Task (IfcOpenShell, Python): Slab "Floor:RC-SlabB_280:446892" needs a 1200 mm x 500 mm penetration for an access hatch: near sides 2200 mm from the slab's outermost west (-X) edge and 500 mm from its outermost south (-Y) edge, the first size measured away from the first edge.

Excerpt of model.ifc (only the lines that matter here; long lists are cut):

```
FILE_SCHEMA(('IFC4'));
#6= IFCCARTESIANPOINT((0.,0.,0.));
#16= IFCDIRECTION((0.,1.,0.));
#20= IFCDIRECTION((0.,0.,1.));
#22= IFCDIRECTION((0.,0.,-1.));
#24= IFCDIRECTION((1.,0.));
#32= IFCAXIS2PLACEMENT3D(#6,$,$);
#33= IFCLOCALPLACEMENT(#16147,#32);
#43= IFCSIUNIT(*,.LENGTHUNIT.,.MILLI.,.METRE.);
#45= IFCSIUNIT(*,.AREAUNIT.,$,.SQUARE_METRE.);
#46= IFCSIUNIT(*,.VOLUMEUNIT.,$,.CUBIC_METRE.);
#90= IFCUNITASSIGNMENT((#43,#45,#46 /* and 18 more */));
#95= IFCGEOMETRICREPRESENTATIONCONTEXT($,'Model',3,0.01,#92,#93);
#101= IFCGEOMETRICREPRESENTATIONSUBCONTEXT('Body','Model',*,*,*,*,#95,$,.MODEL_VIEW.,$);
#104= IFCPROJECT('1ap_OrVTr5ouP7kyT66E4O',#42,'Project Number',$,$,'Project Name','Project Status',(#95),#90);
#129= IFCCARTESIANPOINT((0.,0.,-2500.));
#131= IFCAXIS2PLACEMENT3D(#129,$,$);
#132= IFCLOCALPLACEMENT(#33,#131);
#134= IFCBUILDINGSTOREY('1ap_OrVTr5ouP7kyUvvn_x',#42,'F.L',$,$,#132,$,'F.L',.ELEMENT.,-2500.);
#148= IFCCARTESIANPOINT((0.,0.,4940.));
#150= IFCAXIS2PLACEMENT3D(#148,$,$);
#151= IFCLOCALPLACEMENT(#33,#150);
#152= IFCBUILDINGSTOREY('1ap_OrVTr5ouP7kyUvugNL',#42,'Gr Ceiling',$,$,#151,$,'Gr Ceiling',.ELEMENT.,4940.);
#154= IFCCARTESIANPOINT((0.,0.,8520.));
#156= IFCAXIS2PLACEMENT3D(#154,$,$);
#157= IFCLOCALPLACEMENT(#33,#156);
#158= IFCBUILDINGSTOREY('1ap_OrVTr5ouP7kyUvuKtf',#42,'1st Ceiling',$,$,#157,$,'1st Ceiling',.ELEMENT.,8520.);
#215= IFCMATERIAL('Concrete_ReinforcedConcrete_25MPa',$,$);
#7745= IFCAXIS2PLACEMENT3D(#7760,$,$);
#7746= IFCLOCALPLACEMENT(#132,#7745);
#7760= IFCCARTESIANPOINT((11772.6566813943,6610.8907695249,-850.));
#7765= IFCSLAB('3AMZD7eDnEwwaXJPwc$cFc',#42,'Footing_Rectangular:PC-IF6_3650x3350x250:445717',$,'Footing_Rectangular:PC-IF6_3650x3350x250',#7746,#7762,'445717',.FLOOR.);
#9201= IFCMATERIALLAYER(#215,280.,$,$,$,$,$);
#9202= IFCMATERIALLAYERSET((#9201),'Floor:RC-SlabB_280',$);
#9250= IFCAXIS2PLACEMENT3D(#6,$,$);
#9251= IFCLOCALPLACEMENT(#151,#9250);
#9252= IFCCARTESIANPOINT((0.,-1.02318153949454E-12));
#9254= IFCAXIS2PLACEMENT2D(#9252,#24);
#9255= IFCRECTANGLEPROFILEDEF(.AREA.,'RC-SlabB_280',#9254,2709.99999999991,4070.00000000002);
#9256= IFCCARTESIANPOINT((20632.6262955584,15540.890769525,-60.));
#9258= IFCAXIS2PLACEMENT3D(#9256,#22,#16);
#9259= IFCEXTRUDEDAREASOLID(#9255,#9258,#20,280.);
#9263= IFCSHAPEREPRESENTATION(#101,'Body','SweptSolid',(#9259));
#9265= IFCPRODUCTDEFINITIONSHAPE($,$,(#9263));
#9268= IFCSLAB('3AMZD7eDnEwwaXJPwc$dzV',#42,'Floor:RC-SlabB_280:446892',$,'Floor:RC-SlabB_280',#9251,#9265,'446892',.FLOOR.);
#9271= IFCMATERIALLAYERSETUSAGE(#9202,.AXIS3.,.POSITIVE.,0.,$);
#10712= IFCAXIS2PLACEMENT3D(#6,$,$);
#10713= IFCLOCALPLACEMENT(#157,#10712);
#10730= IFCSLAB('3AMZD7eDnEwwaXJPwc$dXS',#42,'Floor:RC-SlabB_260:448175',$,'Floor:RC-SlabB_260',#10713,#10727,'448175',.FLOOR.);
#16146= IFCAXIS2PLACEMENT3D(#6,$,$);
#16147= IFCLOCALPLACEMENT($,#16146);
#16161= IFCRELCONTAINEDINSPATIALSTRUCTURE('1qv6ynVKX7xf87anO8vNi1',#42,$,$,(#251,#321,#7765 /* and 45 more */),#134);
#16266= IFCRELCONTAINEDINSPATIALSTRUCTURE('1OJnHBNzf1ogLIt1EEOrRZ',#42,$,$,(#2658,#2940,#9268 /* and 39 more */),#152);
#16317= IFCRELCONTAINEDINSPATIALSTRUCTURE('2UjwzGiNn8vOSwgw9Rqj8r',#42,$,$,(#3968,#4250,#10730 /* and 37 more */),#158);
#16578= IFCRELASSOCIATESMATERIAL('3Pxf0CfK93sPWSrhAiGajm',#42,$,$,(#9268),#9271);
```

```python
import numpy as np
import ifcopenshell
import ifcopenshell.api.feature
import ifcopenshell.api.geometry
import ifcopenshell.api.root
import ifcopenshell.geom
import ifcopenshell.util.placement
import ifcopenshell.util.representation
import ifcopenshell.util.shape
import ifcopenshell.util.unit

model = ifcopenshell.open("model.ifc")
unit_scale = ifcopenshell.util.unit.calculate_unit_scale(model)
settings = ifcopenshell.geom.settings()


def volume(element):
    """Net volume in cubic metres, openings subtracted."""
    shape = ifcopenshell.geom.create_shape(settings, element)
    return ifcopenshell.util.shape.get_volume(shape.geometry)


slab = model.by_id(9268)
before = volume(slab)

# Extent in the slab's own axes, in metres. The edges named are its -X and -Y sides.
slab_shape = ifcopenshell.geom.create_shape(settings, slab)
vertices = ifcopenshell.util.shape.get_vertices(slab_shape.geometry)
x_min, y_min, bottom = vertices.min(axis=0)
top = vertices[:, 2].max()

opening = ifcopenshell.api.root.create_entity(model, ifc_class="IfcOpeningElement", name="Access hatch opening", predefined_type="OPENING")
context = ifcopenshell.util.representation.get_context(model, "Model", "Body", "MODEL_VIEW")
width, depth = 1.2, 0.5
outline = [(0.0, 0.0), (width, 0.0), (width, depth), (0.0, depth), (0.0, 0.0)]
# Overshoot both faces by 50 mm so the cut is clean.
shape = ifcopenshell.api.geometry.add_slab_representation(
    model, context=context, depth=top - bottom + 0.1, polyline=outline
)
ifcopenshell.api.geometry.assign_representation(model, product=opening, representation=shape)

matrix = ifcopenshell.util.placement.get_local_placement(slab.ObjectPlacement)
matrix[:, 3] = matrix @ np.append(np.array([x_min + 2.2, y_min + 0.5, bottom - 0.05]) / unit_scale, 1.0)
ifcopenshell.api.geometry.edit_object_placement(model, product=opening, matrix=matrix, is_si=False)
ifcopenshell.api.feature.add_feature(model, feature=opening, element=slab)

after = volume(slab)

print(f"slab volume {before:.3f} -> {after:.3f} m3")

model.write("model_v2.ifc")
```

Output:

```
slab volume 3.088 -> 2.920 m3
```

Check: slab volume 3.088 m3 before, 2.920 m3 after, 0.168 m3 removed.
